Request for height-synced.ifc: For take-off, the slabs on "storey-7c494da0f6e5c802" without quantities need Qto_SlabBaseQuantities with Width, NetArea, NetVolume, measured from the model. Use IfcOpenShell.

First a look at what the model holds.

```python
import ifcopenshell
import ifcopenshell.util.element
import ifcopenshell.util.unit

model = ifcopenshell.open("height-synced.ifc")
print(model.schema)
for unit_type in ("LENGTHUNIT", "AREAUNIT", "VOLUMEUNIT"):
    print(unit_type, ifcopenshell.util.unit.calculate_unit_scale(model, unit_type))
storey = next(s for s in model.by_type("IfcBuildingStorey") if s.Name == "storey-7c494da0f6e5c802")
slabs = [e for e in ifcopenshell.util.element.get_decomposition(storey) if e.is_a("IfcSlab")]
for e in sorted(slabs, key=lambda e: e.id()):
    print(e.id(), e.is_a(), e.Name, list(ifcopenshell.util.element.get_psets(e, qtos_only=True)), sep=" | ")
```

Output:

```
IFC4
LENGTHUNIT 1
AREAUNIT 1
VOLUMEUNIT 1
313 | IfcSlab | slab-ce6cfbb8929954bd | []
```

```python
import ifcopenshell
import ifcopenshell.api.pset
import ifcopenshell.geom
import ifcopenshell.util.element
import ifcopenshell.util.shape
import ifcopenshell.util.unit

model = ifcopenshell.open("height-synced.ifc")
unit_scale = ifcopenshell.util.unit.calculate_unit_scale(model)
area_scale = ifcopenshell.util.unit.calculate_unit_scale(model, "AREAUNIT")
volume_scale = ifcopenshell.util.unit.calculate_unit_scale(model, "VOLUMEUNIT")
settings = ifcopenshell.geom.settings()

storey = next(s for s in model.by_type("IfcBuildingStorey") if s.Name == "storey-7c494da0f6e5c802")
slabs = [e for e in ifcopenshell.util.element.get_decomposition(storey) if e.is_a("IfcSlab")]

for e in sorted(slabs, key=lambda e: e.id()):
    if ifcopenshell.util.element.get_psets(e, qtos_only=True, should_inherit=False):
        continue
    # Geometry comes back in metres, in the element's own axes.
    shape = ifcopenshell.geom.create_shape(settings, e)
    values = {
        "Width": ifcopenshell.util.shape.get_z(shape.geometry) / unit_scale,
        "NetArea": ifcopenshell.util.shape.get_footprint_area(shape.geometry) / area_scale,
        "NetVolume": ifcopenshell.util.shape.get_volume(shape.geometry) / volume_scale,
    }
    qto = ifcopenshell.api.pset.add_qto(model, product=e, name="Qto_SlabBaseQuantities")
    ifcopenshell.api.pset.edit_qto(model, qto=qto, properties=values)
    print(e.id(), {k: round(v, 3) for k, v in values.items()})

model.write("height-synced_v2.ifc")
```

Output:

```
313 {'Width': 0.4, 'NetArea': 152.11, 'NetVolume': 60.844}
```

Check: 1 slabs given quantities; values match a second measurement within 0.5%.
